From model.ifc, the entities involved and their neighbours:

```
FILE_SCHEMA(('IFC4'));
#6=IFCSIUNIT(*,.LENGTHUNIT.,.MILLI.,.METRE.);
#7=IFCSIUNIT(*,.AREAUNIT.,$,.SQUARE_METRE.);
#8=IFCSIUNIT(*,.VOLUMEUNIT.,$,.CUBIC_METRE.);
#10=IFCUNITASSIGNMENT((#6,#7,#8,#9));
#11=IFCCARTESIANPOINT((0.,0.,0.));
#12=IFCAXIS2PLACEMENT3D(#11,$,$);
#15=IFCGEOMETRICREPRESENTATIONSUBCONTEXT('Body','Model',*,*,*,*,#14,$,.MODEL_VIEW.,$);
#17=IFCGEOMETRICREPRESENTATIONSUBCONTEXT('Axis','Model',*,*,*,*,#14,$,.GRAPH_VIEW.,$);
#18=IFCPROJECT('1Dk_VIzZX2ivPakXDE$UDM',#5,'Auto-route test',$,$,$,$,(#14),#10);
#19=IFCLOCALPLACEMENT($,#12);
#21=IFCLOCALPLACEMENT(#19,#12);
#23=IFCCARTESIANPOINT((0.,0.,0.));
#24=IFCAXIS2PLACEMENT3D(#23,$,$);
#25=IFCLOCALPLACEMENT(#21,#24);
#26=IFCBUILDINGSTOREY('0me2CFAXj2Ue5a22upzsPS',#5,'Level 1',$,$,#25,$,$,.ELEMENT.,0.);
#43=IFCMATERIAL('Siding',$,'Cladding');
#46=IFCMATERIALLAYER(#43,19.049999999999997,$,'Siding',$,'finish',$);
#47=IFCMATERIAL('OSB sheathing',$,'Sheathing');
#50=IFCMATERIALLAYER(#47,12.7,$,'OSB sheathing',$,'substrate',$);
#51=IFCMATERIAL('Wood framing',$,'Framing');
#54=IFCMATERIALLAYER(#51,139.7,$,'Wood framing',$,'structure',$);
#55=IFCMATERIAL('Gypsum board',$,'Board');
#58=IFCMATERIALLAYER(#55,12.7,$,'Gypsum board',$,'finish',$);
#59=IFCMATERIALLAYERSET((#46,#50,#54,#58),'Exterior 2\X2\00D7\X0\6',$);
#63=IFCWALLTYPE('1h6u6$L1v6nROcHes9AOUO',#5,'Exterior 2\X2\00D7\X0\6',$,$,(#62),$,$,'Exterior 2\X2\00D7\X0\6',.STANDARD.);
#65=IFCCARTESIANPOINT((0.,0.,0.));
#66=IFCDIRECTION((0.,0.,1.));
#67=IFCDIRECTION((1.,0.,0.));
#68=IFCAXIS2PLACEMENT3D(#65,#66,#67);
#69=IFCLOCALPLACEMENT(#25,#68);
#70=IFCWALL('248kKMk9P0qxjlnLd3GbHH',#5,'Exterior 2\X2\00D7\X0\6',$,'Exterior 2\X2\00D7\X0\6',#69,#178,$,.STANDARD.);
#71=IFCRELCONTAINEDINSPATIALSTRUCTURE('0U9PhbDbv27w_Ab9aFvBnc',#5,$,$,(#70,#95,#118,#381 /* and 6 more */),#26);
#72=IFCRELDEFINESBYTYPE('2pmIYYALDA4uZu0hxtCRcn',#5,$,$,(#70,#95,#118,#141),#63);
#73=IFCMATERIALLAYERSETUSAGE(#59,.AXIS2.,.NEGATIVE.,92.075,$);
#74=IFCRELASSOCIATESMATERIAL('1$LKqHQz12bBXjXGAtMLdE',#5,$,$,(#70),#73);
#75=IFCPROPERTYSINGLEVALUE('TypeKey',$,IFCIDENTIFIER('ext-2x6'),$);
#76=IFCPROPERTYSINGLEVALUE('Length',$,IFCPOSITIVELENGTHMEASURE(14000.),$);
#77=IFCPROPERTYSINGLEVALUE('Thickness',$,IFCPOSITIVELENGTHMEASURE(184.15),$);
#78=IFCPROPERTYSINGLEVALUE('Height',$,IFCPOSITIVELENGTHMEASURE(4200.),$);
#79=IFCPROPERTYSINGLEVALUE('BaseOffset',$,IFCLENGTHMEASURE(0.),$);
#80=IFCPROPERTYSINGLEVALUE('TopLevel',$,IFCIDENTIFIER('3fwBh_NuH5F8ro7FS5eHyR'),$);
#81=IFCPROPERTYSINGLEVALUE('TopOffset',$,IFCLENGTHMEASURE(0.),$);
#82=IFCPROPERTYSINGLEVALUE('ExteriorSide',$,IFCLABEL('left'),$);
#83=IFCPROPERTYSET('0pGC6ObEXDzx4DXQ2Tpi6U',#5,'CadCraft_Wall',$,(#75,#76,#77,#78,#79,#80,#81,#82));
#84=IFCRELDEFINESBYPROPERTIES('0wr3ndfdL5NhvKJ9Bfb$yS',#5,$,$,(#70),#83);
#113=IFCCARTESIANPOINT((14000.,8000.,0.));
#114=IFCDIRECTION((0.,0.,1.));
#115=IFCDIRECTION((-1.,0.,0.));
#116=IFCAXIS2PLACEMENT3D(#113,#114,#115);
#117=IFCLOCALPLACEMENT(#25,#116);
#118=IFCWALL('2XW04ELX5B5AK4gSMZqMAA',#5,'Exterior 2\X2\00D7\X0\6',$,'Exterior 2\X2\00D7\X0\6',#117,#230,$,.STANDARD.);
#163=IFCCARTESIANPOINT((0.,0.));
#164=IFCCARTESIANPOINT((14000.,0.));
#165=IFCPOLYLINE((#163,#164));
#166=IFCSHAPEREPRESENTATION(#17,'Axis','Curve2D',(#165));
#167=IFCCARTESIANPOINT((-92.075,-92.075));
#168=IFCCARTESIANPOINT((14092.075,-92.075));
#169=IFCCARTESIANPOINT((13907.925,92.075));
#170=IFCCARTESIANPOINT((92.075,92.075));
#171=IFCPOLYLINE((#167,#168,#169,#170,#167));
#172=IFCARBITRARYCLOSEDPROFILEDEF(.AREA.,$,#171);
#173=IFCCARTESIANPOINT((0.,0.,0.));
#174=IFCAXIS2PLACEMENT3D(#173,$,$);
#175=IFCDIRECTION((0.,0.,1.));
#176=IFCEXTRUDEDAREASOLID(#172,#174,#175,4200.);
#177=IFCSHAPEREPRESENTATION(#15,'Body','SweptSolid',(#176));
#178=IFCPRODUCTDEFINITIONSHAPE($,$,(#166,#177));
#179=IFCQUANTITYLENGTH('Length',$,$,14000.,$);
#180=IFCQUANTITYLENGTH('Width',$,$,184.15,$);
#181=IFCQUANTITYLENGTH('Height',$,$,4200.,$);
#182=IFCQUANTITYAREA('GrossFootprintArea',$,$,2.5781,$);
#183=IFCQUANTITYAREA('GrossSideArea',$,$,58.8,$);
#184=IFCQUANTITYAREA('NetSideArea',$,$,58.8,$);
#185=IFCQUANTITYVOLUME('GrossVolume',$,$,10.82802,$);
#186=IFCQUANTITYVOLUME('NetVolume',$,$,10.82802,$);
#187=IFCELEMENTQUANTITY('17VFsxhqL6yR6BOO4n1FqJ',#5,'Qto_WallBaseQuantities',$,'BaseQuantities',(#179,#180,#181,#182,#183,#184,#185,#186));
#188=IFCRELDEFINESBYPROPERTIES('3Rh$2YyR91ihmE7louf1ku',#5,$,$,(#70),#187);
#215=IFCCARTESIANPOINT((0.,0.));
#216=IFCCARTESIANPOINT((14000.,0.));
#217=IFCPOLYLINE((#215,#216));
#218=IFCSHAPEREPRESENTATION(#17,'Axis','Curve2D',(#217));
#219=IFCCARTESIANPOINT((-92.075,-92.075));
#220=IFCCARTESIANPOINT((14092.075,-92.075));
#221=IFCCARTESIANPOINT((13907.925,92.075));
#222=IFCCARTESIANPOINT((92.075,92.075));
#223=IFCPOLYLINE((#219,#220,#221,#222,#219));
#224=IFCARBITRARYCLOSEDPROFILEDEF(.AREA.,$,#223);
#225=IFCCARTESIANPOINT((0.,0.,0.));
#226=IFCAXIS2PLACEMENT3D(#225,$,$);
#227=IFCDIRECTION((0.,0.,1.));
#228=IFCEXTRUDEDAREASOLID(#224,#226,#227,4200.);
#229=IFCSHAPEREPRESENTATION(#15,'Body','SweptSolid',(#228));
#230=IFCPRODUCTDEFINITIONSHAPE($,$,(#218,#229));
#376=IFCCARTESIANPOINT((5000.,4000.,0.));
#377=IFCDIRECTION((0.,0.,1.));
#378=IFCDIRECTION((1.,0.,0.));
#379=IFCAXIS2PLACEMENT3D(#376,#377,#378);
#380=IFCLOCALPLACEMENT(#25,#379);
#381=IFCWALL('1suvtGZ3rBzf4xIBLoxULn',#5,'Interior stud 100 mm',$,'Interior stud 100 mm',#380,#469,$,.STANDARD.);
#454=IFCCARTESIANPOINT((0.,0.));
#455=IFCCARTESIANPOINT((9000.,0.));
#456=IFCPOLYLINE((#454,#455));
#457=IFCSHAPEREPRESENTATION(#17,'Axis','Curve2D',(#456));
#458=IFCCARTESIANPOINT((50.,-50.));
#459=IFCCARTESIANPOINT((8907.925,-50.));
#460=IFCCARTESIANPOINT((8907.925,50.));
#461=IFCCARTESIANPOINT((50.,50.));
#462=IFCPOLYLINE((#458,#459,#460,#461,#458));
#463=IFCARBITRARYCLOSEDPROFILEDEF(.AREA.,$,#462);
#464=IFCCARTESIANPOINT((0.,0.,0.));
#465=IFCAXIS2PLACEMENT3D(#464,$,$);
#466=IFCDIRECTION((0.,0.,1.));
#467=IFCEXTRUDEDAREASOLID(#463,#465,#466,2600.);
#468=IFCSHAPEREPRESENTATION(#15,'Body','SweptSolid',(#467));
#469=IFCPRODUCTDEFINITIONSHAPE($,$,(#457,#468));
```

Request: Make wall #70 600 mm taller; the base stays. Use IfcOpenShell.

```python
import ifcopenshell
import ifcopenshell.api.pset
import ifcopenshell.geom
import ifcopenshell.util.element
import ifcopenshell.util.representation
import ifcopenshell.util.shape
import ifcopenshell.util.unit

model = ifcopenshell.open("model.ifc")
unit_scale = ifcopenshell.util.unit.calculate_unit_scale(model)
area_scale = ifcopenshell.util.unit.calculate_unit_scale(model, "AREAUNIT")
volume_scale = ifcopenshell.util.unit.calculate_unit_scale(model, "VOLUMEUNIT")
settings = ifcopenshell.geom.settings()


def volume(element):
    """Net volume in cubic metres, openings subtracted."""
    shape = ifcopenshell.geom.create_shape(settings, element)
    return ifcopenshell.util.shape.get_volume(shape.geometry)


wall = model.by_guid("248kKMk9P0qxjlnLd3GbHH")
before = volume(wall)

body = ifcopenshell.util.representation.get_representation(wall, "Model", "Body")
solid = body.Items[0]
old_height = solid.Depth
solid.Depth += 0.6 / unit_scale
after = volume(wall)
thickness = 0.1842  # wall thickness in metres

# Update the stored height, areas and volumes.
pset = model.by_id(ifcopenshell.util.element.get_pset(wall, "CadCraft_Wall", should_inherit=False)["id"])
ifcopenshell.api.pset.edit_pset(model, pset=pset, properties={
    "Height": model.create_entity("IfcPositiveLengthMeasure", solid.Depth),
})
qto = model.by_id(ifcopenshell.util.element.get_pset(wall, "Qto_WallBaseQuantities", should_inherit=False)["id"])
ifcopenshell.api.pset.edit_qto(model, qto=qto, properties={
    "Height": solid.Depth,
    "GrossSideArea": ifcopenshell.util.element.get_pset(wall, "Qto_WallBaseQuantities", "GrossSideArea") * solid.Depth / old_height,
    "NetSideArea": after / thickness / area_scale,
    "GrossVolume": ifcopenshell.util.element.get_pset(wall, "Qto_WallBaseQuantities", "GrossVolume") * solid.Depth / old_height,
    "NetVolume": after / volume_scale,
})

print(f"height {old_height:g} -> {solid.Depth:g}, volume {before:.3f} -> {after:.3f} m3")

model.write("model_rev.ifc")
```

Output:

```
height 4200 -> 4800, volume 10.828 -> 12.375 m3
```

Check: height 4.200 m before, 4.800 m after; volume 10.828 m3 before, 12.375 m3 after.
